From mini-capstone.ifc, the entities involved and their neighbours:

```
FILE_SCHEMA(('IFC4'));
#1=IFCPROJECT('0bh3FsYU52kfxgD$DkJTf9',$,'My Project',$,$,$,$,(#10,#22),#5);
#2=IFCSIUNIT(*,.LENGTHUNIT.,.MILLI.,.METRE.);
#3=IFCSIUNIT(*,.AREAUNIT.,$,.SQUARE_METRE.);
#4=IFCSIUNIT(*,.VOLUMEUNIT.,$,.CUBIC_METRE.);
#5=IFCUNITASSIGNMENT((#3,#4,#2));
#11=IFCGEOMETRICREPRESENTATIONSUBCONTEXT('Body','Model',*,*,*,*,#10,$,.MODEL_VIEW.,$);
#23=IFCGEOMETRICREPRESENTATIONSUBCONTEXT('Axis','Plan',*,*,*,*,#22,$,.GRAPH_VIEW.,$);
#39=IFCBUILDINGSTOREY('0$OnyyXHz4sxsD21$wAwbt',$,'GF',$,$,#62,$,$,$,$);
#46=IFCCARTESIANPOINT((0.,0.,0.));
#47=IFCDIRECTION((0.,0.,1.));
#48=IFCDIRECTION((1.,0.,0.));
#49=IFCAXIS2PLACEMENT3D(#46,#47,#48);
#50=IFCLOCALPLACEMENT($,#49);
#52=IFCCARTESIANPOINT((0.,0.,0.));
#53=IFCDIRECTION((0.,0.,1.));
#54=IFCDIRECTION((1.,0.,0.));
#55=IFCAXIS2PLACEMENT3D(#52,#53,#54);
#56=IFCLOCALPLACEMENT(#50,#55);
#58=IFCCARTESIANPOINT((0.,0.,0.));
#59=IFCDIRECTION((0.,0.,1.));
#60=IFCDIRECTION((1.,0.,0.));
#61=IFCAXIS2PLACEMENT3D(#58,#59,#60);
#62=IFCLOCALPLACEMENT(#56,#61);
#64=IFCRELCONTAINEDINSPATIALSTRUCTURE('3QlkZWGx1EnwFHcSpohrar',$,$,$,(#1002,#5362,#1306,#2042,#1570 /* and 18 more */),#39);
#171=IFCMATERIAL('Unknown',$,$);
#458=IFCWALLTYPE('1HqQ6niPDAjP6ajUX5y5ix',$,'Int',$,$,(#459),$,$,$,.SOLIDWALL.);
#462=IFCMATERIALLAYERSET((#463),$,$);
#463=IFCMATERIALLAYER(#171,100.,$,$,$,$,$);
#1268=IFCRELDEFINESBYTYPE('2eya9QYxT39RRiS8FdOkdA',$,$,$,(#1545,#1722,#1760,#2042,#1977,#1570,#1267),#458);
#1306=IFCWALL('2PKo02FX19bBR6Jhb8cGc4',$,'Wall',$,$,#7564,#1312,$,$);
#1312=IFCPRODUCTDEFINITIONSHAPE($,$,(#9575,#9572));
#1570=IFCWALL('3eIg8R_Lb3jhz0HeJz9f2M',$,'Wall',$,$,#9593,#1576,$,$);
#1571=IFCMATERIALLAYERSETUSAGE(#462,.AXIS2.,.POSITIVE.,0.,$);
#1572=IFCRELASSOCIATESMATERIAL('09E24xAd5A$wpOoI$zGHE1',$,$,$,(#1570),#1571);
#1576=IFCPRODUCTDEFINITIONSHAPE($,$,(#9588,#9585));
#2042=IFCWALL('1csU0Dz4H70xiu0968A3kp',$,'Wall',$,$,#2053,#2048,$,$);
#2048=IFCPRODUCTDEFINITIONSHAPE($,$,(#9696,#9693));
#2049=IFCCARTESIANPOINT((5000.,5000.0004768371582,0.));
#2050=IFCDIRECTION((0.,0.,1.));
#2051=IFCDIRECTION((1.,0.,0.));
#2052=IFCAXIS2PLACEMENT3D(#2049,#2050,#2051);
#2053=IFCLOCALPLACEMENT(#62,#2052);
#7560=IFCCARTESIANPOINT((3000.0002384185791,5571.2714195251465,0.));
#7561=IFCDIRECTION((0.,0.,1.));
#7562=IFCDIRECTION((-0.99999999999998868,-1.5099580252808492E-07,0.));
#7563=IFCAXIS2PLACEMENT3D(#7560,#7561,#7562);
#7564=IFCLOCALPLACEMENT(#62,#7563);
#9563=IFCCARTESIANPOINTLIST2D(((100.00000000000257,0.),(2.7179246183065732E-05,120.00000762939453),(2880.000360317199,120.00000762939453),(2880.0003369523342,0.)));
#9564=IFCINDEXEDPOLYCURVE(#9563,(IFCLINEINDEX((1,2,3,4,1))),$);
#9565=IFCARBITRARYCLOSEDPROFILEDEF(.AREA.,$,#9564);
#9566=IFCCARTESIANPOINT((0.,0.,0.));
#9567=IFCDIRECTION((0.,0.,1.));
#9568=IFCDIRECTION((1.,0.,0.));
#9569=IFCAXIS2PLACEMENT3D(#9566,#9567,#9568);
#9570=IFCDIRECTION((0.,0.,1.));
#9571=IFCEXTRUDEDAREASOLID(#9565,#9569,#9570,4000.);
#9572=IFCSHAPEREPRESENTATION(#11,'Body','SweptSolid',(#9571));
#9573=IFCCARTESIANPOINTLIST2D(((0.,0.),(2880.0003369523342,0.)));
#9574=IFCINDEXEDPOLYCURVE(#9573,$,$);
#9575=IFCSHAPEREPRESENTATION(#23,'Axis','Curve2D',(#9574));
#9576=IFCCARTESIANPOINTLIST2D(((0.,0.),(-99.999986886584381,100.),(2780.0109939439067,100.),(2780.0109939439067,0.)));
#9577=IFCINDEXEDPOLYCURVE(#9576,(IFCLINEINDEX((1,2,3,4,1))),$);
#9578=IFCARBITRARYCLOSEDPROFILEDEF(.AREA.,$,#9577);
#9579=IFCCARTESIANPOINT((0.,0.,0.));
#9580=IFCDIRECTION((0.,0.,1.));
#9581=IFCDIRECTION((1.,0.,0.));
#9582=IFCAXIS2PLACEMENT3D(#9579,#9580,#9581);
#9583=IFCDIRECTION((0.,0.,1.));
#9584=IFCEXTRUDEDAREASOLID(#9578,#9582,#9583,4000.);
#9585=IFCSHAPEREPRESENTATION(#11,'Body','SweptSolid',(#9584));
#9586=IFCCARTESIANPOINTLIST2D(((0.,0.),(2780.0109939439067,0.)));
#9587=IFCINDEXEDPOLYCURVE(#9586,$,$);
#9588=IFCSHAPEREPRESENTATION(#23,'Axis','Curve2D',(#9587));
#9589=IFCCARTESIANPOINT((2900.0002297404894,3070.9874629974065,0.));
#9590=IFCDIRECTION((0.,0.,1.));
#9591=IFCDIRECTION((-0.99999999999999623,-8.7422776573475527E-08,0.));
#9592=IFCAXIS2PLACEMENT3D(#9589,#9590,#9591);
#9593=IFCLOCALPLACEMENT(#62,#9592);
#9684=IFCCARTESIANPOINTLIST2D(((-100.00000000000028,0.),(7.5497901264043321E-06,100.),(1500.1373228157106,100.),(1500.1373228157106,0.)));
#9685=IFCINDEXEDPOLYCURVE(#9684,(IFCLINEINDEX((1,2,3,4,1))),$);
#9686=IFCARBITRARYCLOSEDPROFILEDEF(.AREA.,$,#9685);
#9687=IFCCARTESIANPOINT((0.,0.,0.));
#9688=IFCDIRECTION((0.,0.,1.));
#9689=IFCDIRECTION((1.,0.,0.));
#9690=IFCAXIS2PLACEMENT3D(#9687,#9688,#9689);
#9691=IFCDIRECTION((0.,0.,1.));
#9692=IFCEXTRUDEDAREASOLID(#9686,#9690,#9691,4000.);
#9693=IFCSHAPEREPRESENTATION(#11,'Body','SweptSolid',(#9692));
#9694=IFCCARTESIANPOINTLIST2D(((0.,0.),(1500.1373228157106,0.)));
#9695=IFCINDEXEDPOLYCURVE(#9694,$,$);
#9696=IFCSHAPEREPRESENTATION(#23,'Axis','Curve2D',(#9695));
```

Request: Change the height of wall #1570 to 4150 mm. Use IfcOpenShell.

```python
import ifcopenshell
import ifcopenshell.geom
import ifcopenshell.util.representation
import ifcopenshell.util.shape

model = ifcopenshell.open("mini-capstone.ifc")
settings = ifcopenshell.geom.settings()


def volume(element):
    """Net volume in cubic metres, openings subtracted."""
    shape = ifcopenshell.geom.create_shape(settings, element)
    return ifcopenshell.util.shape.get_volume(shape.geometry)


wall = model.by_guid("3eIg8R_Lb3jhz0HeJz9f2M")
before = volume(wall)

body = ifcopenshell.util.representation.get_representation(wall, "Model", "Body")
solid = body.Items[0]
old_height = solid.Depth
solid.Depth = 4150.0
after = volume(wall)

print(f"height {old_height:g} -> {solid.Depth:g}, volume {before:.3f} -> {after:.3f} m3")

model.write("mini-capstone_updated.ifc")
```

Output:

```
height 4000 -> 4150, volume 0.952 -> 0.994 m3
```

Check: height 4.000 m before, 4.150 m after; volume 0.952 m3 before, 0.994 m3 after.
